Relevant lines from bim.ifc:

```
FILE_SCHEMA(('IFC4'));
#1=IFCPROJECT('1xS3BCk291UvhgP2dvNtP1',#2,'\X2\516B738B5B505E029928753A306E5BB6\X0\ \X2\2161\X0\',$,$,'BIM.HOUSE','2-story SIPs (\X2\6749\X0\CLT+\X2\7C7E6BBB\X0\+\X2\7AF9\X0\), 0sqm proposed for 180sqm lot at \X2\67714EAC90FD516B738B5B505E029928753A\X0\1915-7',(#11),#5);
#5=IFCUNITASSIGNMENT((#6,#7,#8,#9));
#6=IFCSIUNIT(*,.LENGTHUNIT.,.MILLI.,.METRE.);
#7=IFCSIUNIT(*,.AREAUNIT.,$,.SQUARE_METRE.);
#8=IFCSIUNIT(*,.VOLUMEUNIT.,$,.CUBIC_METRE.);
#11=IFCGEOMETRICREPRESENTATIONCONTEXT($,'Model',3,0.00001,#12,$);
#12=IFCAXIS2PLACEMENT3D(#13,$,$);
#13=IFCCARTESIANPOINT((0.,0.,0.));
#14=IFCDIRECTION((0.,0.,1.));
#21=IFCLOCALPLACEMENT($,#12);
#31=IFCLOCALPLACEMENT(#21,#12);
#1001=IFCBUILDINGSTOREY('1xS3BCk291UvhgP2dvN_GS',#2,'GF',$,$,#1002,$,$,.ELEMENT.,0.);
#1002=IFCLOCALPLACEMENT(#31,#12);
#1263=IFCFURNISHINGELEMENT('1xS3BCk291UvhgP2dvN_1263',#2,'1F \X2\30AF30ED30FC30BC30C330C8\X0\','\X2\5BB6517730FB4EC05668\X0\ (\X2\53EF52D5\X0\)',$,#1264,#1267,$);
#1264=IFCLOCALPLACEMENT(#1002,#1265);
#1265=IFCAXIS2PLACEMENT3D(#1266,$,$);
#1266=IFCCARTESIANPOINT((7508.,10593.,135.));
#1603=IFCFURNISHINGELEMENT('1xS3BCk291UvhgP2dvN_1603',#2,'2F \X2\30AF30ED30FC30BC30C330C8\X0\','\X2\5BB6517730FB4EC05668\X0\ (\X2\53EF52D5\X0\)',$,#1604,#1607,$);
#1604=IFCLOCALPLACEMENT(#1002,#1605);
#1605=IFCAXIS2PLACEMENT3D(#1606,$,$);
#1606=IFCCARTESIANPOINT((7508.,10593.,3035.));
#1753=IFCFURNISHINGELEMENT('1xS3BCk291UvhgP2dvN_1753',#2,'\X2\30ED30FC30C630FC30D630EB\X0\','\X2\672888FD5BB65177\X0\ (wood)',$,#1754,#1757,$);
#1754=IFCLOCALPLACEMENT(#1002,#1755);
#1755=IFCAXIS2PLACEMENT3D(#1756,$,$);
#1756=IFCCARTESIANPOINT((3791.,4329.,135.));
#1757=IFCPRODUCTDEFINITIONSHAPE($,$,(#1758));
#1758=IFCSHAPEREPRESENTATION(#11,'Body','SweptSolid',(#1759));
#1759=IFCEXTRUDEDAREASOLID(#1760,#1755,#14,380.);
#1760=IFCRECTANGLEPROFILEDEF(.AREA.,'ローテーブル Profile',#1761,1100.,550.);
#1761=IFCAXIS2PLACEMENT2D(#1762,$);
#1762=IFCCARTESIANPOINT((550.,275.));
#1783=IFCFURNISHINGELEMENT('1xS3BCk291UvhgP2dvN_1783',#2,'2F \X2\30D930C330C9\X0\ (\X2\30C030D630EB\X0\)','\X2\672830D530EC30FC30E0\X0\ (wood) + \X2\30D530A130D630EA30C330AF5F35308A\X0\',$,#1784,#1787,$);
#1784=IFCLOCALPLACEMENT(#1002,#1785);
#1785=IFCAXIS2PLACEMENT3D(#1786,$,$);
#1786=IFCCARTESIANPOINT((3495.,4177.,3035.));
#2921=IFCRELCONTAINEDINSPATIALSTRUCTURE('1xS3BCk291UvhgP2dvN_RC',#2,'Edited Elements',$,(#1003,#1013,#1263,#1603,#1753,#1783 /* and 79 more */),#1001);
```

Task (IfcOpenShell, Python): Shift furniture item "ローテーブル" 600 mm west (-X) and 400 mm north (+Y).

```python
import ifcopenshell
import ifcopenshell.api.geometry
import ifcopenshell.util.placement

model = ifcopenshell.open("bim.ifc")

item = model.by_guid("1xS3BCk291UvhgP2dvN_1753")
matrix = ifcopenshell.util.placement.get_local_placement(item.ObjectPlacement)
matrix[0, 3] -= 600.0
matrix[1, 3] += 400.0
ifcopenshell.api.geometry.edit_object_placement(model, product=item, matrix=matrix, is_si=False)

print(ifcopenshell.util.placement.get_local_placement(item.ObjectPlacement).round(3) + 0.0)

model.write("bim_rev.ifc")
```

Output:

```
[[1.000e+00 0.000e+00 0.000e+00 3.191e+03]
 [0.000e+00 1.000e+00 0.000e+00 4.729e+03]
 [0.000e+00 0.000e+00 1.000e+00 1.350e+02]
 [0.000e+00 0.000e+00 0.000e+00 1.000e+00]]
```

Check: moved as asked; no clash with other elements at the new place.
